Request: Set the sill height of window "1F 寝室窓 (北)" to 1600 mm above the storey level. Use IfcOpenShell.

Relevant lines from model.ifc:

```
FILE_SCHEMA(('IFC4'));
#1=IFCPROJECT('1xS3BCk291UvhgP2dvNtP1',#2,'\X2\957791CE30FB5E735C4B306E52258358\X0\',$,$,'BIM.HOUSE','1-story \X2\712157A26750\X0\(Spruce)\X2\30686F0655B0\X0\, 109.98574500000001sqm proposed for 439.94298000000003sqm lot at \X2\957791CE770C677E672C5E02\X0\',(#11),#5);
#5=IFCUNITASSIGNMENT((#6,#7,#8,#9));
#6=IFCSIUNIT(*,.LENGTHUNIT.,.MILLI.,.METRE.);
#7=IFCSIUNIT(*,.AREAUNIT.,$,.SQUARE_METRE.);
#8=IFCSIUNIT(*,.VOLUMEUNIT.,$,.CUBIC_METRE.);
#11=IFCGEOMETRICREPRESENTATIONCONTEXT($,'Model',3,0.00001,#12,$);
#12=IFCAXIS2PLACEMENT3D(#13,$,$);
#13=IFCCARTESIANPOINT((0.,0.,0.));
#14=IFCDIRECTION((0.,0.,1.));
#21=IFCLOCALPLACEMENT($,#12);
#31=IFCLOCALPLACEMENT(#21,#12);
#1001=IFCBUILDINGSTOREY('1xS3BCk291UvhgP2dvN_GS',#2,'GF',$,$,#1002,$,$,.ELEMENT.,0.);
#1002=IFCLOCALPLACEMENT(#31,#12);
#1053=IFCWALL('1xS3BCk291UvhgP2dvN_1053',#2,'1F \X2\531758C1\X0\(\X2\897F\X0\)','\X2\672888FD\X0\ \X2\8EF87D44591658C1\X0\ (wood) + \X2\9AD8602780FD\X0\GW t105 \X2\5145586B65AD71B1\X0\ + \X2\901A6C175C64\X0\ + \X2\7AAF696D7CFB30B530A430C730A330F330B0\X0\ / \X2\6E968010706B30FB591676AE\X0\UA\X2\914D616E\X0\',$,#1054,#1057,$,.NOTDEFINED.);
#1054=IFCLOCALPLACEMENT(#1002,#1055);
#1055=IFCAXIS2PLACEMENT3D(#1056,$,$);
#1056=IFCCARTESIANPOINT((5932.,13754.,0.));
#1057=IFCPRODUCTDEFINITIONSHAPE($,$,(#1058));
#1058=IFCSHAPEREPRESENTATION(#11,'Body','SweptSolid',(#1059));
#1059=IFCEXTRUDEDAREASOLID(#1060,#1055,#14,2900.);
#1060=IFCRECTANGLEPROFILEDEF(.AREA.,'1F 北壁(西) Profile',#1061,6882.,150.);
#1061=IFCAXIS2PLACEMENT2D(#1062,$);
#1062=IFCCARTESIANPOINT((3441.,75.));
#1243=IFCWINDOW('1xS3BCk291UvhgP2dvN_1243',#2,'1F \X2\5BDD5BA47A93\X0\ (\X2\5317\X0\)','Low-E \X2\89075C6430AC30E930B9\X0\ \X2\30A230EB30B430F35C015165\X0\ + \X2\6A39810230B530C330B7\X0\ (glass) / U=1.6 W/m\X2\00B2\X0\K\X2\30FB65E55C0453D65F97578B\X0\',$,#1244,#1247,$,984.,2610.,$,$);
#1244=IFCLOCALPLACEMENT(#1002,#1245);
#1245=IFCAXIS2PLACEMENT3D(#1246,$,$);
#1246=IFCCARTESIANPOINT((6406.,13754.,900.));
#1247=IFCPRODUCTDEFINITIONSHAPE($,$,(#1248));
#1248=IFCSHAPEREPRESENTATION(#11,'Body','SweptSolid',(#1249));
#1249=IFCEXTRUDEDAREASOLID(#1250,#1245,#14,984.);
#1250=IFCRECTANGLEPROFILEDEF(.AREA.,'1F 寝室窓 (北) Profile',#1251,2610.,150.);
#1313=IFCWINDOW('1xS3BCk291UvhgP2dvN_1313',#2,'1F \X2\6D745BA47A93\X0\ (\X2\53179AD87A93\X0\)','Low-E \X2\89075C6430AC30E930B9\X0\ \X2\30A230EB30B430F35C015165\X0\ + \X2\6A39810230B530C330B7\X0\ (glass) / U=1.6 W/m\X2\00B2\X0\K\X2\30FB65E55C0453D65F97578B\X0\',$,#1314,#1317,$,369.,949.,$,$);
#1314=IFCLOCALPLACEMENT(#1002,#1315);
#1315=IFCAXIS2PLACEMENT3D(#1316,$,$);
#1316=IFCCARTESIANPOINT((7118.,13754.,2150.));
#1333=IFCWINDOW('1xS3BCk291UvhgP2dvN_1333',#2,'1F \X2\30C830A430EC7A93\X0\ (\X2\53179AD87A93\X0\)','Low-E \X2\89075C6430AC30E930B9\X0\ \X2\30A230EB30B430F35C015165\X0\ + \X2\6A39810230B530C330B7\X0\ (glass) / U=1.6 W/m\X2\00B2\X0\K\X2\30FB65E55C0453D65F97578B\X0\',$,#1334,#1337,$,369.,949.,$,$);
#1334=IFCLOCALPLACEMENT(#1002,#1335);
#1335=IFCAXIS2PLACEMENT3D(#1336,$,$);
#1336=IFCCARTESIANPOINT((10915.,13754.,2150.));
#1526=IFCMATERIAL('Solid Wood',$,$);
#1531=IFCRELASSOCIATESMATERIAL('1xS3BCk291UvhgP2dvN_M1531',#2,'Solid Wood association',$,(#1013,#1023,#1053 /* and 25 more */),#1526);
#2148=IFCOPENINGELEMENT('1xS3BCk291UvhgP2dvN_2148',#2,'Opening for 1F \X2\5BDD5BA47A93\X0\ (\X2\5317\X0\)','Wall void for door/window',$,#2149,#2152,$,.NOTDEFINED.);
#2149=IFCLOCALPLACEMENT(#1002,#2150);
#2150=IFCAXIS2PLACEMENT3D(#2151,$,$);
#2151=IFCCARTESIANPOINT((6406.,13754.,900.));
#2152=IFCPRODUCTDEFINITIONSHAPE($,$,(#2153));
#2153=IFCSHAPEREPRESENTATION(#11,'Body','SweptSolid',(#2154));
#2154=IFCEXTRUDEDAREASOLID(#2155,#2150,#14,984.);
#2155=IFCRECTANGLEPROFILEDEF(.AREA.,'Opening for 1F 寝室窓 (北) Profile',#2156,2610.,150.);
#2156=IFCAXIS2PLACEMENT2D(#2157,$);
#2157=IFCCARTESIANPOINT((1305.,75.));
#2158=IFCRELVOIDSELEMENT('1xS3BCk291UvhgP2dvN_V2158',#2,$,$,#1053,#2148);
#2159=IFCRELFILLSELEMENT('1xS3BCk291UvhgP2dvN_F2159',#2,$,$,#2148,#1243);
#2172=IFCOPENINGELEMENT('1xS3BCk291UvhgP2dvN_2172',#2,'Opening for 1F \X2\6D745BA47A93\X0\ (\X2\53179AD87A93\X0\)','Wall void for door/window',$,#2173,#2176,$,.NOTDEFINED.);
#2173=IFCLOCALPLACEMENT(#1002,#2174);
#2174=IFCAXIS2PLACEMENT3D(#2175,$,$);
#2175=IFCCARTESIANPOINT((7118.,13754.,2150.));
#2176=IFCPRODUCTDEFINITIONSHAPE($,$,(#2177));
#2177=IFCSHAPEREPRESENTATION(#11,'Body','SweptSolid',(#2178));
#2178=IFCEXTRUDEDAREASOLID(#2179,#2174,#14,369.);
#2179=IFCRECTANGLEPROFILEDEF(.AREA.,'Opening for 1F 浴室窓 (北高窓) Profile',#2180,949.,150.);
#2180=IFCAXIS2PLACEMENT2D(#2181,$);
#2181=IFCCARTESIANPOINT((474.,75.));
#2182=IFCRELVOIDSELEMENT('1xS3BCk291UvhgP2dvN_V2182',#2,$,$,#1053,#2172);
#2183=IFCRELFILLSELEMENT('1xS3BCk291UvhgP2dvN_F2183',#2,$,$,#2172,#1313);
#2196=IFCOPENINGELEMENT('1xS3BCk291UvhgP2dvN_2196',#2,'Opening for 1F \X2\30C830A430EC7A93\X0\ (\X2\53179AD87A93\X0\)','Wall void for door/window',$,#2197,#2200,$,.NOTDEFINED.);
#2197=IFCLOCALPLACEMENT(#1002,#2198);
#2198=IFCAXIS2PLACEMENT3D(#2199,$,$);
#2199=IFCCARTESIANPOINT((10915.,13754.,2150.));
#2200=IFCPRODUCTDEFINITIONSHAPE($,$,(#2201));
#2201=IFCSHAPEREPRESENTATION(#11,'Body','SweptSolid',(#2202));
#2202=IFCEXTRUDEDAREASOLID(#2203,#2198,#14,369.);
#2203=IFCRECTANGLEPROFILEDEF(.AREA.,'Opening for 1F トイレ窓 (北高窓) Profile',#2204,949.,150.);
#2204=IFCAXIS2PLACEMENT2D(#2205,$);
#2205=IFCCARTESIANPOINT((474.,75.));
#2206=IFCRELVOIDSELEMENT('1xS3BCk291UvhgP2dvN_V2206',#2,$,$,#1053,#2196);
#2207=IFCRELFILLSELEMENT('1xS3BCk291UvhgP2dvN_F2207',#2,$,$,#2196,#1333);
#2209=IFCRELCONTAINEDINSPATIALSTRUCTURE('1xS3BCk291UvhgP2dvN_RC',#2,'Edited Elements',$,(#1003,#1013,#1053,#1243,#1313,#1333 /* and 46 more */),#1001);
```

```python
import numpy as np
import ifcopenshell
import ifcopenshell.api.geometry
import ifcopenshell.geom
import ifcopenshell.util.element
import ifcopenshell.util.placement
import ifcopenshell.util.shape
import ifcopenshell.util.unit

model = ifcopenshell.open("model.ifc")
unit_scale = ifcopenshell.util.unit.calculate_unit_scale(model)

window = model.by_guid("1xS3BCk291UvhgP2dvN_1243")
opening = window.FillsVoids[0].RelatingOpeningElement
storey = ifcopenshell.util.element.get_container(window, ifc_class="IfcBuildingStorey")
level = ifcopenshell.util.placement.get_local_placement(storey.ObjectPlacement)[2, 3]

# The opening's origin need not be at the sill, so measure its lowest point.
shape = ifcopenshell.geom.create_shape(ifcopenshell.geom.settings(), opening)
bottom = ifcopenshell.util.shape.get_shape_bottom_elevation(shape, shape.geometry) / unit_scale
dz = level + 1.6 / unit_scale - bottom

shift = np.array([0.0, 0.0, dz])
# The window is not placed relative to its opening, so move both.
for product in (opening, window):
    matrix = ifcopenshell.util.placement.get_local_placement(product.ObjectPlacement)
    matrix[:3, 3] += shift
    ifcopenshell.api.geometry.edit_object_placement(model, product=product, matrix=matrix, is_si=False)

print(f"moved by {dz * unit_scale:+.3f} m")

model.write("model_updated.ifc")
```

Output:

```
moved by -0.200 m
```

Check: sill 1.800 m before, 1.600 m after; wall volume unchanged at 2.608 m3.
